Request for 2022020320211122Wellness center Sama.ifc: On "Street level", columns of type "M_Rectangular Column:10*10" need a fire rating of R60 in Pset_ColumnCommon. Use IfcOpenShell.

First a look at what the model holds.

```python
import ifcopenshell
import ifcopenshell.util.element

model = ifcopenshell.open("2022020320211122Wellness center Sama.ifc")
print(model.schema)
storey = next(s for s in model.by_type("IfcBuildingStorey") if s.Name == "Street level")
columns = [e for e in ifcopenshell.util.element.get_decomposition(storey) if e.is_a("IfcColumn")]
seen = {}
for e in columns:
    element_type = ifcopenshell.util.element.get_type(e)
    key = (element_type.Name if element_type != e and element_type else None, ifcopenshell.util.element.get_pset(e, "Pset_ColumnCommon", "FireRating"))
    seen[key] = seen.get(key, 0) + 1
for (name, value), count in sorted(seen.items(), key=str):
    print(count, "x", name, "|", value)
```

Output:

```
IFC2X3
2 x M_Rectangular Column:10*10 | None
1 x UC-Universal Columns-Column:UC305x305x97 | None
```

```python
import ifcopenshell
import ifcopenshell.api.pset
import ifcopenshell.util.element

model = ifcopenshell.open("2022020320211122Wellness center Sama.ifc")

storey = next(s for s in model.by_type("IfcBuildingStorey") if s.Name == "Street level")
columns = [e for e in ifcopenshell.util.element.get_decomposition(storey) if e.is_a("IfcColumn")]

count = 0
for e in columns:
    element_type = ifcopenshell.util.element.get_type(e)
    if element_type in (None, e) or element_type.Name != "M_Rectangular Column:10*10":
        continue
    # add_pset returns the element's existing set when there is one.
    pset = ifcopenshell.api.pset.add_pset(model, product=e, name="Pset_ColumnCommon")
    ifcopenshell.api.pset.edit_pset(model, pset=pset, properties={"FireRating": "R60"})
    count += 1

print(count, "columns updated")

model.write("2022020320211122Wellness center Sama_edited.ifc")
```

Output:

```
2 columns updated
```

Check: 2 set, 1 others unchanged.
